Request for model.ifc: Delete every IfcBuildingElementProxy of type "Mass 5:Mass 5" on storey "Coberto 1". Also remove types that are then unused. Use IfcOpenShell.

First a look at what the model holds.

```python
import ifcopenshell
import ifcopenshell.util.element

model = ifcopenshell.open("model.ifc")
print(model.schema)
storey = next(s for s in model.by_type("IfcBuildingStorey") if s.Name == "Coberto 1")
proxies = [e for e in ifcopenshell.util.element.get_decomposition(storey) if e.is_a("IfcBuildingElementProxy")]
seen = {}
for e in proxies:
    element_type = ifcopenshell.util.element.get_type(e)
    name = element_type.Name if element_type not in (None, e) else None
    seen[name] = seen.get(name, 0) + 1
for name, count in sorted(seen.items(), key=str):
    print(count, "x", name)
```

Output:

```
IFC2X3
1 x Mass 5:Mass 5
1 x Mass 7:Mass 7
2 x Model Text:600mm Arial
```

```python
import ifcopenshell
import ifcopenshell.api.root
import ifcopenshell.util.element

model = ifcopenshell.open("model.ifc")

storey = next(s for s in model.by_type("IfcBuildingStorey") if s.Name == "Coberto 1")
proxies = [e for e in ifcopenshell.util.element.get_decomposition(storey) if e.is_a("IfcBuildingElementProxy")]
targets = [e for e in proxies if (t := ifcopenshell.util.element.get_type(e)) not in (None, e) and t.Name == "Mass 5:Mass 5"]
types = {ifcopenshell.util.element.get_type(e) for e in targets} - {None, *targets}

for e in targets:
    ifcopenshell.api.root.remove_product(model, product=e)
print(len(targets), "removed")

unused = [t for t in types if not ifcopenshell.util.element.get_types(t)]
for t in unused:
    ifcopenshell.api.root.remove_product(model, product=t)
print(len(unused), "unused types removed")

model.write("model_edited.ifc")
```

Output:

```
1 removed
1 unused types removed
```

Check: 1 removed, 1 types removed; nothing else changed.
